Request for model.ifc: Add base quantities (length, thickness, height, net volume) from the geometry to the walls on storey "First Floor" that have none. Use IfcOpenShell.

First a look at what the model holds.

```python
import ifcopenshell
import ifcopenshell.util.element
import ifcopenshell.util.unit

model = ifcopenshell.open("model.ifc")
print(model.schema)
for unit_type in ("LENGTHUNIT", "AREAUNIT", "VOLUMEUNIT"):
    print(unit_type, ifcopenshell.util.unit.calculate_unit_scale(model, unit_type))
storey = next(s for s in model.by_type("IfcBuildingStorey") if s.Name == "First Floor")
walls = [e for e in ifcopenshell.util.element.get_decomposition(storey) if e.is_a("IfcWall")]
for e in sorted(walls, key=lambda e: e.id()):
    print(e.id(), e.is_a(), e.Name, list(ifcopenshell.util.element.get_psets(e, qtos_only=True)), sep=" | ")
```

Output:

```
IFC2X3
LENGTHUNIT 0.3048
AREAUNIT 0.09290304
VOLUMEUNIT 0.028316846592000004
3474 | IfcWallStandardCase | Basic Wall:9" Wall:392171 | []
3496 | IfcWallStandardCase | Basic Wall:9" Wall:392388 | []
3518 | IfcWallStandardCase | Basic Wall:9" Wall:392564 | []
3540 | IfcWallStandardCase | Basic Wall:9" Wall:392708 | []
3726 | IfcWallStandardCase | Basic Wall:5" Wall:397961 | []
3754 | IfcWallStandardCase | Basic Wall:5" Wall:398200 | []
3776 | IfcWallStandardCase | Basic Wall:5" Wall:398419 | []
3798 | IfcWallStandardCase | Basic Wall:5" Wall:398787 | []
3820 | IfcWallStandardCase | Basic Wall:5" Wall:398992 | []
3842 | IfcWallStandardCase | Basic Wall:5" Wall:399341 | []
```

```python
import ifcopenshell
import ifcopenshell.api.pset
import ifcopenshell.geom
import ifcopenshell.util.element
import ifcopenshell.util.shape
import ifcopenshell.util.unit

model = ifcopenshell.open("model.ifc")
unit_scale = ifcopenshell.util.unit.calculate_unit_scale(model)
volume_scale = ifcopenshell.util.unit.calculate_unit_scale(model, "VOLUMEUNIT")
settings = ifcopenshell.geom.settings()

storey = next(s for s in model.by_type("IfcBuildingStorey") if s.Name == "First Floor")
walls = [e for e in ifcopenshell.util.element.get_decomposition(storey) if e.is_a("IfcWall")]

for e in sorted(walls, key=lambda e: e.id()):
    if ifcopenshell.util.element.get_psets(e, qtos_only=True, should_inherit=False):
        continue
    # Geometry comes back in metres, in the element's own axes.
    shape = ifcopenshell.geom.create_shape(settings, e)
    values = {
        "Length": ifcopenshell.util.shape.get_x(shape.geometry) / unit_scale,
        "Width": ifcopenshell.util.shape.get_y(shape.geometry) / unit_scale,
        "Height": ifcopenshell.util.shape.get_z(shape.geometry) / unit_scale,
        "NetVolume": ifcopenshell.util.shape.get_volume(shape.geometry) / volume_scale,
    }
    qto = ifcopenshell.api.pset.add_qto(model, product=e, name="BaseQuantities")
    ifcopenshell.api.pset.edit_qto(model, qto=qto, properties=values)
    print(e.id(), {k: round(v, 3) for k, v in values.items()})

model.write("model_edited.ifc")
```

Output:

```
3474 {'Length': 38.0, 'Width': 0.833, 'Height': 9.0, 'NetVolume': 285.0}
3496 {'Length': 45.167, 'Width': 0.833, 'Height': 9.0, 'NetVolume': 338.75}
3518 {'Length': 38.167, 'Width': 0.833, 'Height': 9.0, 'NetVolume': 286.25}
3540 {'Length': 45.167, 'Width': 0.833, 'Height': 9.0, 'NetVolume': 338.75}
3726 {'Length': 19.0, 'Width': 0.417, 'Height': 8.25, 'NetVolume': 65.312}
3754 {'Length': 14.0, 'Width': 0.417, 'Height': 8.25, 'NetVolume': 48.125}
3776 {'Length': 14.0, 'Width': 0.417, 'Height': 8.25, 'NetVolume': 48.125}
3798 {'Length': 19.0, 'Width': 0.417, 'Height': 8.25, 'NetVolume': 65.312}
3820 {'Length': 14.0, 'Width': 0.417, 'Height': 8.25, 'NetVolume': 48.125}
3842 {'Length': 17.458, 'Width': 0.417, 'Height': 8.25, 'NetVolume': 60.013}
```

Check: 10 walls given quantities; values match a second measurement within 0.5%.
